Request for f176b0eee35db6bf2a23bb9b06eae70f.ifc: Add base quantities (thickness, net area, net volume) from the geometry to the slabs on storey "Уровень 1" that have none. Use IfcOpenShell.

First a look at what the model holds.

```python
import ifcopenshell
import ifcopenshell.util.element
import ifcopenshell.util.unit

model = ifcopenshell.open("f176b0eee35db6bf2a23bb9b06eae70f.ifc")
print(model.schema)
for unit_type in ("LENGTHUNIT", "AREAUNIT", "VOLUMEUNIT"):
    print(unit_type, ifcopenshell.util.unit.calculate_unit_scale(model, unit_type))
storey = next(s for s in model.by_type("IfcBuildingStorey") if s.Name == "Уровень 1")
slabs = [e for e in ifcopenshell.util.element.get_decomposition(storey) if e.is_a("IfcSlab")]
for e in sorted(slabs, key=lambda e: e.id()):
    print(e.id(), e.is_a(), e.Name, list(ifcopenshell.util.element.get_psets(e, qtos_only=True)), sep=" | ")
```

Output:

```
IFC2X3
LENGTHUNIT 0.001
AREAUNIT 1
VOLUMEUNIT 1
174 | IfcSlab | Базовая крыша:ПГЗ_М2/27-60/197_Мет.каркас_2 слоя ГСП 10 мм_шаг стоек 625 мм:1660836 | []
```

```python
import ifcopenshell
import ifcopenshell.api.pset
import ifcopenshell.geom
import ifcopenshell.util.element
import ifcopenshell.util.shape
import ifcopenshell.util.unit

model = ifcopenshell.open("f176b0eee35db6bf2a23bb9b06eae70f.ifc")
unit_scale = ifcopenshell.util.unit.calculate_unit_scale(model)
area_scale = ifcopenshell.util.unit.calculate_unit_scale(model, "AREAUNIT")
volume_scale = ifcopenshell.util.unit.calculate_unit_scale(model, "VOLUMEUNIT")
settings = ifcopenshell.geom.settings()

storey = next(s for s in model.by_type("IfcBuildingStorey") if s.Name == "Уровень 1")
slabs = [e for e in ifcopenshell.util.element.get_decomposition(storey) if e.is_a("IfcSlab")]

for e in sorted(slabs, key=lambda e: e.id()):
    if ifcopenshell.util.element.get_psets(e, qtos_only=True, should_inherit=False):
        continue
    # Geometry comes back in metres, in the element's own axes.
    shape = ifcopenshell.geom.create_shape(settings, e)
    values = {
        "Width": ifcopenshell.util.shape.get_z(shape.geometry) / unit_scale,
        "NetArea": ifcopenshell.util.shape.get_footprint_area(shape.geometry) / area_scale,
        "NetVolume": ifcopenshell.util.shape.get_volume(shape.geometry) / volume_scale,
    }
    qto = ifcopenshell.api.pset.add_qto(model, product=e, name="BaseQuantities")
    ifcopenshell.api.pset.edit_qto(model, qto=qto, properties=values)
    print(e.id(), {k: round(v, 3) for k, v in values.items()})

model.write("f176b0eee35db6bf2a23bb9b06eae70f_v2.ifc")
```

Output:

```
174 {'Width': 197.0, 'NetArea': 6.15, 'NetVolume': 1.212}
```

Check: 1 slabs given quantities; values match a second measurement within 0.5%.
